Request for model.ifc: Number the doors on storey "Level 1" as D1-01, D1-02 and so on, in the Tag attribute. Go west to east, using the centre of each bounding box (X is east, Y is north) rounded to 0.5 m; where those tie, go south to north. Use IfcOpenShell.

First a look at what the model holds.

```python
import ifcopenshell
import ifcopenshell.util.element
import ifcopenshell.util.placement

model = ifcopenshell.open("model.ifc")
print(model.schema)
storey = next(s for s in model.by_type("IfcBuildingStorey") if s.Name == "Level 1")
doors = [e for e in ifcopenshell.util.element.get_decomposition(storey) if e.is_a("IfcDoor")]
for e in sorted(doors, key=lambda e: e.id()):
    origin = ifcopenshell.util.placement.get_local_placement(e.ObjectPlacement)[:3, 3]
    print(e.id(), e.Tag, e.Name, origin.round(2) + 0.0, sep=" | ")
```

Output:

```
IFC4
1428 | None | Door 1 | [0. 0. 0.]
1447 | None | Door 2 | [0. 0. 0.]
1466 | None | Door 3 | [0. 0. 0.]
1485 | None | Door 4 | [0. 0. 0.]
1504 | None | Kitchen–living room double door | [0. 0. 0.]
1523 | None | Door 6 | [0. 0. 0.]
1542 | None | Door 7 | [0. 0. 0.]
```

```python
import ifcopenshell
import ifcopenshell.geom
import ifcopenshell.util.element
import ifcopenshell.util.shape

model = ifcopenshell.open("model.ifc")
settings = ifcopenshell.geom.settings()
settings.set("use-world-coords", True)


def centre(element):
    shape = ifcopenshell.geom.create_shape(settings, element)
    return ifcopenshell.util.shape.get_bbox_centroid(shape.geometry)


storey = next(s for s in model.by_type("IfcBuildingStorey") if s.Name == "Level 1")
doors = [e for e in ifcopenshell.util.element.get_decomposition(storey) if e.is_a("IfcDoor")]

# Insertion points can sit at a corner or the storey origin, so sort by the geometry (in metres).
centres = {e: centre(e) for e in doors}
doors.sort(key=lambda e: (round(centres[e][0] / 0.5), centres[e][1]))

for i, e in enumerate(doors, start=1):
    number = f"D1-{i:02d}"
    e.Tag = number
    print(e.id(), number)

model.write("model_updated.ifc")
```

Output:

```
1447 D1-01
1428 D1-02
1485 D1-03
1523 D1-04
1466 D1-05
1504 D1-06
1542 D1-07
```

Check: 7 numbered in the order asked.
